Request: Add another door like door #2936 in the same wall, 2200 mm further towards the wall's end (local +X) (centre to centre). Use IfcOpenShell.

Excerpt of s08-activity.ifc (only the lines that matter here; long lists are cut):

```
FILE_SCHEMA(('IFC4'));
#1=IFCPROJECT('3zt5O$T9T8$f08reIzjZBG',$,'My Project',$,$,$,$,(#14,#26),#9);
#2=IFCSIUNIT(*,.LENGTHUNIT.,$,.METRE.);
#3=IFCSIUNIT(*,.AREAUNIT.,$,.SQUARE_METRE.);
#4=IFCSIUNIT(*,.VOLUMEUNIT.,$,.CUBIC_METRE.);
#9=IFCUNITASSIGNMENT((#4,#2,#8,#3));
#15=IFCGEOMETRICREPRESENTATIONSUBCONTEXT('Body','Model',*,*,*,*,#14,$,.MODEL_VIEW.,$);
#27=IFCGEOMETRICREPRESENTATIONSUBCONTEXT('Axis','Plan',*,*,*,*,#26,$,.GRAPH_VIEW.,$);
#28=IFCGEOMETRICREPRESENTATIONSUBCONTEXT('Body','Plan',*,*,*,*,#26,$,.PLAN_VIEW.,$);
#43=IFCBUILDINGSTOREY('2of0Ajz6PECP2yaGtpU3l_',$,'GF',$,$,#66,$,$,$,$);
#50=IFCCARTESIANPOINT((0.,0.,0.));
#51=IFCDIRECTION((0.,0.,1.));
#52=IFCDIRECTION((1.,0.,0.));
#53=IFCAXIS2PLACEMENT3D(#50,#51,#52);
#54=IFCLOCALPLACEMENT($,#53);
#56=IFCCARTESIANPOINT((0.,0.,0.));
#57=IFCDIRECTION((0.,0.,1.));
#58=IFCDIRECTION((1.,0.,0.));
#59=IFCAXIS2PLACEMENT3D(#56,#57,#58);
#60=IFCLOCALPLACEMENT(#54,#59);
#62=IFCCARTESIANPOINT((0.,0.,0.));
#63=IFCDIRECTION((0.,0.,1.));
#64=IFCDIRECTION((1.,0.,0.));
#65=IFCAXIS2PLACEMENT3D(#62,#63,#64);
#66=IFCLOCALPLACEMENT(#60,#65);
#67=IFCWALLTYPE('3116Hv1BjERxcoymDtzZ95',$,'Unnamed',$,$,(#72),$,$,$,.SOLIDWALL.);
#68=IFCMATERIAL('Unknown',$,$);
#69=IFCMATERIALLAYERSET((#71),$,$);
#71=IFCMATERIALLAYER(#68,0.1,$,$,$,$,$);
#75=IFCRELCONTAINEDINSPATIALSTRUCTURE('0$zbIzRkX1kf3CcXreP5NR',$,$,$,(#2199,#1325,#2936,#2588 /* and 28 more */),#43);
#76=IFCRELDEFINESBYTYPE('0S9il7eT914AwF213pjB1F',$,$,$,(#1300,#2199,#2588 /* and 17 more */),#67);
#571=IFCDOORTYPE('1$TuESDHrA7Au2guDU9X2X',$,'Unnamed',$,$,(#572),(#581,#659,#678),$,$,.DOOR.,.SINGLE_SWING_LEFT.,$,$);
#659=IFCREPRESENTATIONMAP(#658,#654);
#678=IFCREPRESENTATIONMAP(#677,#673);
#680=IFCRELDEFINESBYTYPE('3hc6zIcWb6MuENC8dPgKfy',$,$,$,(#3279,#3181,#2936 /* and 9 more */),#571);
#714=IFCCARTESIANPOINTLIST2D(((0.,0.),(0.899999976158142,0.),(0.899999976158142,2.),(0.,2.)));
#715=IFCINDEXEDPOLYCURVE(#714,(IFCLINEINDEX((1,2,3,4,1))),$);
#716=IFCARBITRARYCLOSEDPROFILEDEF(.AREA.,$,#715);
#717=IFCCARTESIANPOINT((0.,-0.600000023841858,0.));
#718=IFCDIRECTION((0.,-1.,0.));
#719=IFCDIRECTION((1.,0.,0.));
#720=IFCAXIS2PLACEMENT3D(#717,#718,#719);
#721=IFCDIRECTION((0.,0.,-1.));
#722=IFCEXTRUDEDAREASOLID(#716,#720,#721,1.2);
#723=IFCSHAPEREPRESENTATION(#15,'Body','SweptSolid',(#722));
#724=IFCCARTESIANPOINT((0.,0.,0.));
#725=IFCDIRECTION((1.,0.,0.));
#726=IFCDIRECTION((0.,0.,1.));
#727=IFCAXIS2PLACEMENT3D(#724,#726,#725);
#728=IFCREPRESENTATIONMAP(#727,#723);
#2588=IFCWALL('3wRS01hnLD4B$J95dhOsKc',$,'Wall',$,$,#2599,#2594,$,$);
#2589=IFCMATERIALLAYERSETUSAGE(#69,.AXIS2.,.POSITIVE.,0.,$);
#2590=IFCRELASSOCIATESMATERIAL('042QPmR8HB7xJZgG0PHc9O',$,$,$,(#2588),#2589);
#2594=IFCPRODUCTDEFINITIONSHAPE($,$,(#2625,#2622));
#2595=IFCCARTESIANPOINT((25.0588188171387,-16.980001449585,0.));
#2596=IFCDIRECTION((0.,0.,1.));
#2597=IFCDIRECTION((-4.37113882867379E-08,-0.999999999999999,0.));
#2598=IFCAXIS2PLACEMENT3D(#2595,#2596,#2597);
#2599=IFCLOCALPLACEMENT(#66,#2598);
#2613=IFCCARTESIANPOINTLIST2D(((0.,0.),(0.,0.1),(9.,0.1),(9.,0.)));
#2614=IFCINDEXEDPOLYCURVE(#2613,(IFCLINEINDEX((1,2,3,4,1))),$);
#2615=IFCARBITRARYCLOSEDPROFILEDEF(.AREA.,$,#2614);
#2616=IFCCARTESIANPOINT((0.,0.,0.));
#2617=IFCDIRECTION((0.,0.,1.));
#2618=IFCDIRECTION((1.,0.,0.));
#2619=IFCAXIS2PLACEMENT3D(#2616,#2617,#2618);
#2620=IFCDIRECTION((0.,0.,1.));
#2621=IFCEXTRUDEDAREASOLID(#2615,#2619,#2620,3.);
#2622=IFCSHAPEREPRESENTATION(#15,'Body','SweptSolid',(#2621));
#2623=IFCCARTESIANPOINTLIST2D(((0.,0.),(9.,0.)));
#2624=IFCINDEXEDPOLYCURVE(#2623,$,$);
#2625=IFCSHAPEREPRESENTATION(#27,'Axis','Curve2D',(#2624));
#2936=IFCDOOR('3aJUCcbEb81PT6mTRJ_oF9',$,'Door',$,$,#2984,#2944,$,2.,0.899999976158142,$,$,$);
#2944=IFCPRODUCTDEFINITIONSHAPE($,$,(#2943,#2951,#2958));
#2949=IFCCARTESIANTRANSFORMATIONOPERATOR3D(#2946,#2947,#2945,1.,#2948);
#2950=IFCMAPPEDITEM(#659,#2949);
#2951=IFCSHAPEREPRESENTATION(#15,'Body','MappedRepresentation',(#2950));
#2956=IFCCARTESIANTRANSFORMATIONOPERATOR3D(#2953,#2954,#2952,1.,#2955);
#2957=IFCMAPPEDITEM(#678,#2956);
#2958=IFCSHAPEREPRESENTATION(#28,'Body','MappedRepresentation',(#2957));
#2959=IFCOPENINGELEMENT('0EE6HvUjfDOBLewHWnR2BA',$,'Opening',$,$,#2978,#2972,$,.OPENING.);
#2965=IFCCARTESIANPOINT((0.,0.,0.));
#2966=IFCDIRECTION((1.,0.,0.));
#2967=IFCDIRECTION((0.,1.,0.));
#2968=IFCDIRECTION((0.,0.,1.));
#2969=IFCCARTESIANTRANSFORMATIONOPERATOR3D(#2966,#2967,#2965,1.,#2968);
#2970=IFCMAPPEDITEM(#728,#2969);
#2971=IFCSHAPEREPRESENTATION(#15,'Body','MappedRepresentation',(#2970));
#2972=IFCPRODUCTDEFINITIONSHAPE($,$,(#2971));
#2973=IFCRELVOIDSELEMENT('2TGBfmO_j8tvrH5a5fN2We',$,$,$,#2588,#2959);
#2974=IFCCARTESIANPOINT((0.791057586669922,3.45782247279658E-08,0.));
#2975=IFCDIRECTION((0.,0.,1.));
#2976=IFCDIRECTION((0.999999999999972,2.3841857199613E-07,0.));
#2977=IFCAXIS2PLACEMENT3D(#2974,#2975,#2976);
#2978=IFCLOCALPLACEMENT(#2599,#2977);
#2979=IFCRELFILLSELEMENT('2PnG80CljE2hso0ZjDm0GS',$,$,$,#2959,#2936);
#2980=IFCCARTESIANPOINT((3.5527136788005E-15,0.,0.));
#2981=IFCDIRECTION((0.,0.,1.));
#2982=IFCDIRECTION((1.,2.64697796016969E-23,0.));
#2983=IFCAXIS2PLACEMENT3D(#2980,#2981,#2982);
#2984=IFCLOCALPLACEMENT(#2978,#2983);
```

```python
import ifcopenshell
import ifcopenshell.api.feature
import ifcopenshell.api.geometry
import ifcopenshell.api.root
import ifcopenshell.geom
import ifcopenshell.util.element
import ifcopenshell.util.placement
import ifcopenshell.util.shape

model = ifcopenshell.open("s08-activity.ifc")
settings = ifcopenshell.geom.settings()


def volume(element):
    """Net volume in cubic metres, openings subtracted."""
    shape = ifcopenshell.geom.create_shape(settings, element)
    return ifcopenshell.util.shape.get_volume(shape.geometry)


door = model.by_guid("3aJUCcbEb81PT6mTRJ_oF9")
opening = door.FillsVoids[0].RelatingOpeningElement
wall = opening.VoidsElements[0].RelatingBuildingElement
before = volume(wall)
shift = ifcopenshell.util.placement.get_local_placement(wall.ObjectPlacement)[:3, 0] * 2.2

# copy_class copies the void relationship, type, container and properties, but no geometry.
new_opening = ifcopenshell.api.root.copy_class(model, product=opening)
new_opening.Representation = ifcopenshell.util.element.copy_deep(
    model, opening.Representation, exclude=["IfcGeometricRepresentationContext", "IfcRepresentationMap"]
)
new_door = ifcopenshell.api.root.copy_class(model, product=door)
new_door.Representation = ifcopenshell.util.element.copy_deep(
    model, door.Representation, exclude=["IfcGeometricRepresentationContext", "IfcRepresentationMap"]
)
ifcopenshell.api.feature.add_filling(model, opening=new_opening, element=new_door)

for old, new in ((opening, new_opening), (door, new_door)):
    matrix = ifcopenshell.util.placement.get_local_placement(old.ObjectPlacement)
    matrix[:3, 3] += shift
    ifcopenshell.api.geometry.edit_object_placement(model, product=new, matrix=matrix, is_si=False)

after = volume(wall)

print(f"wall volume {before:.3f} -> {after:.3f} m3")

model.write("s08-activity_rev.ifc")
```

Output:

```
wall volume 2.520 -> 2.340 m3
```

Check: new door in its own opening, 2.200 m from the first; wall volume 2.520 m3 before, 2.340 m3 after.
